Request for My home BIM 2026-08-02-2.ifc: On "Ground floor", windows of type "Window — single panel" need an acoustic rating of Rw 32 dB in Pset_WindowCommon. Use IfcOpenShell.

First a look at what the model holds.

```python
import ifcopenshell
import ifcopenshell.util.element

model = ifcopenshell.open("My home BIM 2026-08-02-2.ifc")
print(model.schema)
storey = next(s for s in model.by_type("IfcBuildingStorey") if s.Name == "Ground floor")
windows = [e for e in ifcopenshell.util.element.get_decomposition(storey) if e.is_a("IfcWindow")]
seen = {}
for e in windows:
    element_type = ifcopenshell.util.element.get_type(e)
    key = (element_type.Name if element_type != e and element_type else None, ifcopenshell.util.element.get_pset(e, "Pset_WindowCommon", "AcousticRating"))
    seen[key] = seen.get(key, 0) + 1
for (name, value), count in sorted(seen.items(), key=str):
    print(count, "x", name, "|", value)
```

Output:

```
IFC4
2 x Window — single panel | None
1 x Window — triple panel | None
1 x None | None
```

```python
import ifcopenshell
import ifcopenshell.api.pset
import ifcopenshell.util.element

model = ifcopenshell.open("My home BIM 2026-08-02-2.ifc")

storey = next(s for s in model.by_type("IfcBuildingStorey") if s.Name == "Ground floor")
windows = [e for e in ifcopenshell.util.element.get_decomposition(storey) if e.is_a("IfcWindow")]

count = 0
for e in windows:
    element_type = ifcopenshell.util.element.get_type(e)
    if element_type in (None, e) or element_type.Name != "Window — single panel":
        continue
    # add_pset returns the element's existing set when there is one.
    pset = ifcopenshell.api.pset.add_pset(model, product=e, name="Pset_WindowCommon")
    ifcopenshell.api.pset.edit_pset(model, pset=pset, properties={"AcousticRating": "Rw 32 dB"})
    count += 1

print(count, "windows updated")

model.write("My home BIM 2026-08-02-2-out.ifc")
```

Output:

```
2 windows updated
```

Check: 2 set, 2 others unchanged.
